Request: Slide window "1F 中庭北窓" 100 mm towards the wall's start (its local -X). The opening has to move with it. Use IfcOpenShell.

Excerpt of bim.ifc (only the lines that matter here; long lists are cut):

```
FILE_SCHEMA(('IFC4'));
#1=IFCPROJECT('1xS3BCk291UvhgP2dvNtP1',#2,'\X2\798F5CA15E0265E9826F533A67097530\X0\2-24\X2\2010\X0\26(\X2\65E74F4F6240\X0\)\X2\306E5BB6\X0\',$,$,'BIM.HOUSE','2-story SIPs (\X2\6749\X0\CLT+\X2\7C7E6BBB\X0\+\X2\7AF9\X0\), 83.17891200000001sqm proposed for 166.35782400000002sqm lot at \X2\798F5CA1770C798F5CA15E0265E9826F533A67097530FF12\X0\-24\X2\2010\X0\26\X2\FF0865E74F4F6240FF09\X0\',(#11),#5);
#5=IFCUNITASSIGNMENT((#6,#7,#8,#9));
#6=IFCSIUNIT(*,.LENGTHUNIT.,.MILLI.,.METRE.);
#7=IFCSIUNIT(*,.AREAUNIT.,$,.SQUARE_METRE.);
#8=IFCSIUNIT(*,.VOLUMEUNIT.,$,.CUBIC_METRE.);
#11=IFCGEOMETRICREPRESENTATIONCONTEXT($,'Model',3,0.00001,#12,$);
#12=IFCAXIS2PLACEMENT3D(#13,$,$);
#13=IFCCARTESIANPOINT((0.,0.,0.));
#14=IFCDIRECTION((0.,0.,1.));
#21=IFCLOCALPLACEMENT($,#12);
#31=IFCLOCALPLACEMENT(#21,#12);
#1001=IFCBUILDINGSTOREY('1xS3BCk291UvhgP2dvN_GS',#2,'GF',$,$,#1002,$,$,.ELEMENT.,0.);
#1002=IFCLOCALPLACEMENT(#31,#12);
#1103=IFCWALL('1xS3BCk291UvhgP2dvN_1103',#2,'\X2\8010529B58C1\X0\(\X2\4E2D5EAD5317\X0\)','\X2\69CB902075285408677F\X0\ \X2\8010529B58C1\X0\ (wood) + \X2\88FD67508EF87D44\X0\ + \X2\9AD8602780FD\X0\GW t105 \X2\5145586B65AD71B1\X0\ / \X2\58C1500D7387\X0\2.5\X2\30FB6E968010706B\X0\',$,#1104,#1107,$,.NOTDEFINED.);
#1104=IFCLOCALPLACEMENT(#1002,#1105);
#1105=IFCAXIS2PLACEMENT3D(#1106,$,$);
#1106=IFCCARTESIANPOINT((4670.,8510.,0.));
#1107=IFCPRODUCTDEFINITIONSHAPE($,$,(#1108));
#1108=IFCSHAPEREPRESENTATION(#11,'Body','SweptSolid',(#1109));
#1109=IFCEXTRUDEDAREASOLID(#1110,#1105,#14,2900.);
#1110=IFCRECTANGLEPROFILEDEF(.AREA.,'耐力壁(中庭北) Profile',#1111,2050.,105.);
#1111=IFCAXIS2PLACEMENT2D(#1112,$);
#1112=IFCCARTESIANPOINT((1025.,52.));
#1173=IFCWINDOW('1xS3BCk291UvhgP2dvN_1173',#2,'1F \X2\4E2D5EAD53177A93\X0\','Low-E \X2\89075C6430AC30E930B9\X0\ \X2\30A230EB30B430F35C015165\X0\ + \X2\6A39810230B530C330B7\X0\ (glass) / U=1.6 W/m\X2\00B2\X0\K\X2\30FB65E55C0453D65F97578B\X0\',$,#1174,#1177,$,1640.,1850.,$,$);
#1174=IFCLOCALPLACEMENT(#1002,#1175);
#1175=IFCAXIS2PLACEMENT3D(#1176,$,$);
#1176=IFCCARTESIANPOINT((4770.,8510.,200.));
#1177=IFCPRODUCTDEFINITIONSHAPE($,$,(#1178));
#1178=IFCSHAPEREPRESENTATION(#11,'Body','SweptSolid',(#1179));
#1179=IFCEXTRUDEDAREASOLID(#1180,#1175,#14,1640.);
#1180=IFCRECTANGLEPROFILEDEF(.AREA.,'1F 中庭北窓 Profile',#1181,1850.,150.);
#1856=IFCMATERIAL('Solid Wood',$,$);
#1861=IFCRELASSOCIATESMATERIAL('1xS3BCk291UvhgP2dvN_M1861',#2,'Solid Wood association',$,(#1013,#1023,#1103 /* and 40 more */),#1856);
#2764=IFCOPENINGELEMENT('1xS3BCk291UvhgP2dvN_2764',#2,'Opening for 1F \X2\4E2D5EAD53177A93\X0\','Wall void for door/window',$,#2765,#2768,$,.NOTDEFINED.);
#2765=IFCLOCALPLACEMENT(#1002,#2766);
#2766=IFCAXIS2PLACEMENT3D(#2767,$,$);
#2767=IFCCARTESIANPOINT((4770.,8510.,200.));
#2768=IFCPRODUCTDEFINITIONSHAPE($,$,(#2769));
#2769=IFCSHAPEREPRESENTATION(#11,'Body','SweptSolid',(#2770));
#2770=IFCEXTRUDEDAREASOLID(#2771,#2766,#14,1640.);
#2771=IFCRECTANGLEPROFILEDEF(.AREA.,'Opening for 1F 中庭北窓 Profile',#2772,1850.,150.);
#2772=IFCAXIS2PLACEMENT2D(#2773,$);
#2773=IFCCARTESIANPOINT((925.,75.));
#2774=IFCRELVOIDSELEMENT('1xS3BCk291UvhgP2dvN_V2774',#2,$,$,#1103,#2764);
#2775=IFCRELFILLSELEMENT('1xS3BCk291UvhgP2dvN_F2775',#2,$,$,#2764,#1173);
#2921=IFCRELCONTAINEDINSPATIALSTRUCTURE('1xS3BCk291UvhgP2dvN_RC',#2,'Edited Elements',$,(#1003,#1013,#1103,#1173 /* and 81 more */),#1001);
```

```python
import ifcopenshell
import ifcopenshell.api.geometry
import ifcopenshell.util.placement
import ifcopenshell.util.unit

model = ifcopenshell.open("bim.ifc")
unit_scale = ifcopenshell.util.unit.calculate_unit_scale(model)

window = model.by_id(1173)
opening = window.FillsVoids[0].RelatingOpeningElement
wall = opening.VoidsElements[0].RelatingBuildingElement

wall_matrix = ifcopenshell.util.placement.get_local_placement(wall.ObjectPlacement)
shift = wall_matrix[:3, 0] * -0.1 / unit_scale
before = ifcopenshell.util.placement.get_local_placement(window.ObjectPlacement)[:3, 3].copy()

# The window is not placed relative to its opening, so move both.
for product in (opening, window):
    matrix = ifcopenshell.util.placement.get_local_placement(product.ObjectPlacement)
    matrix[:3, 3] += shift
    ifcopenshell.api.geometry.edit_object_placement(model, product=product, matrix=matrix, is_si=False)

after = ifcopenshell.util.placement.get_local_placement(window.ObjectPlacement)[:3, 3]
print("window moved by", (after - before).round(3) + 0.0)

model.write("bim_updated.ifc")
```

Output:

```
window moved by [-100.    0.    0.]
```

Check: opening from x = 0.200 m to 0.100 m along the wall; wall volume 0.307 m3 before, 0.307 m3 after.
